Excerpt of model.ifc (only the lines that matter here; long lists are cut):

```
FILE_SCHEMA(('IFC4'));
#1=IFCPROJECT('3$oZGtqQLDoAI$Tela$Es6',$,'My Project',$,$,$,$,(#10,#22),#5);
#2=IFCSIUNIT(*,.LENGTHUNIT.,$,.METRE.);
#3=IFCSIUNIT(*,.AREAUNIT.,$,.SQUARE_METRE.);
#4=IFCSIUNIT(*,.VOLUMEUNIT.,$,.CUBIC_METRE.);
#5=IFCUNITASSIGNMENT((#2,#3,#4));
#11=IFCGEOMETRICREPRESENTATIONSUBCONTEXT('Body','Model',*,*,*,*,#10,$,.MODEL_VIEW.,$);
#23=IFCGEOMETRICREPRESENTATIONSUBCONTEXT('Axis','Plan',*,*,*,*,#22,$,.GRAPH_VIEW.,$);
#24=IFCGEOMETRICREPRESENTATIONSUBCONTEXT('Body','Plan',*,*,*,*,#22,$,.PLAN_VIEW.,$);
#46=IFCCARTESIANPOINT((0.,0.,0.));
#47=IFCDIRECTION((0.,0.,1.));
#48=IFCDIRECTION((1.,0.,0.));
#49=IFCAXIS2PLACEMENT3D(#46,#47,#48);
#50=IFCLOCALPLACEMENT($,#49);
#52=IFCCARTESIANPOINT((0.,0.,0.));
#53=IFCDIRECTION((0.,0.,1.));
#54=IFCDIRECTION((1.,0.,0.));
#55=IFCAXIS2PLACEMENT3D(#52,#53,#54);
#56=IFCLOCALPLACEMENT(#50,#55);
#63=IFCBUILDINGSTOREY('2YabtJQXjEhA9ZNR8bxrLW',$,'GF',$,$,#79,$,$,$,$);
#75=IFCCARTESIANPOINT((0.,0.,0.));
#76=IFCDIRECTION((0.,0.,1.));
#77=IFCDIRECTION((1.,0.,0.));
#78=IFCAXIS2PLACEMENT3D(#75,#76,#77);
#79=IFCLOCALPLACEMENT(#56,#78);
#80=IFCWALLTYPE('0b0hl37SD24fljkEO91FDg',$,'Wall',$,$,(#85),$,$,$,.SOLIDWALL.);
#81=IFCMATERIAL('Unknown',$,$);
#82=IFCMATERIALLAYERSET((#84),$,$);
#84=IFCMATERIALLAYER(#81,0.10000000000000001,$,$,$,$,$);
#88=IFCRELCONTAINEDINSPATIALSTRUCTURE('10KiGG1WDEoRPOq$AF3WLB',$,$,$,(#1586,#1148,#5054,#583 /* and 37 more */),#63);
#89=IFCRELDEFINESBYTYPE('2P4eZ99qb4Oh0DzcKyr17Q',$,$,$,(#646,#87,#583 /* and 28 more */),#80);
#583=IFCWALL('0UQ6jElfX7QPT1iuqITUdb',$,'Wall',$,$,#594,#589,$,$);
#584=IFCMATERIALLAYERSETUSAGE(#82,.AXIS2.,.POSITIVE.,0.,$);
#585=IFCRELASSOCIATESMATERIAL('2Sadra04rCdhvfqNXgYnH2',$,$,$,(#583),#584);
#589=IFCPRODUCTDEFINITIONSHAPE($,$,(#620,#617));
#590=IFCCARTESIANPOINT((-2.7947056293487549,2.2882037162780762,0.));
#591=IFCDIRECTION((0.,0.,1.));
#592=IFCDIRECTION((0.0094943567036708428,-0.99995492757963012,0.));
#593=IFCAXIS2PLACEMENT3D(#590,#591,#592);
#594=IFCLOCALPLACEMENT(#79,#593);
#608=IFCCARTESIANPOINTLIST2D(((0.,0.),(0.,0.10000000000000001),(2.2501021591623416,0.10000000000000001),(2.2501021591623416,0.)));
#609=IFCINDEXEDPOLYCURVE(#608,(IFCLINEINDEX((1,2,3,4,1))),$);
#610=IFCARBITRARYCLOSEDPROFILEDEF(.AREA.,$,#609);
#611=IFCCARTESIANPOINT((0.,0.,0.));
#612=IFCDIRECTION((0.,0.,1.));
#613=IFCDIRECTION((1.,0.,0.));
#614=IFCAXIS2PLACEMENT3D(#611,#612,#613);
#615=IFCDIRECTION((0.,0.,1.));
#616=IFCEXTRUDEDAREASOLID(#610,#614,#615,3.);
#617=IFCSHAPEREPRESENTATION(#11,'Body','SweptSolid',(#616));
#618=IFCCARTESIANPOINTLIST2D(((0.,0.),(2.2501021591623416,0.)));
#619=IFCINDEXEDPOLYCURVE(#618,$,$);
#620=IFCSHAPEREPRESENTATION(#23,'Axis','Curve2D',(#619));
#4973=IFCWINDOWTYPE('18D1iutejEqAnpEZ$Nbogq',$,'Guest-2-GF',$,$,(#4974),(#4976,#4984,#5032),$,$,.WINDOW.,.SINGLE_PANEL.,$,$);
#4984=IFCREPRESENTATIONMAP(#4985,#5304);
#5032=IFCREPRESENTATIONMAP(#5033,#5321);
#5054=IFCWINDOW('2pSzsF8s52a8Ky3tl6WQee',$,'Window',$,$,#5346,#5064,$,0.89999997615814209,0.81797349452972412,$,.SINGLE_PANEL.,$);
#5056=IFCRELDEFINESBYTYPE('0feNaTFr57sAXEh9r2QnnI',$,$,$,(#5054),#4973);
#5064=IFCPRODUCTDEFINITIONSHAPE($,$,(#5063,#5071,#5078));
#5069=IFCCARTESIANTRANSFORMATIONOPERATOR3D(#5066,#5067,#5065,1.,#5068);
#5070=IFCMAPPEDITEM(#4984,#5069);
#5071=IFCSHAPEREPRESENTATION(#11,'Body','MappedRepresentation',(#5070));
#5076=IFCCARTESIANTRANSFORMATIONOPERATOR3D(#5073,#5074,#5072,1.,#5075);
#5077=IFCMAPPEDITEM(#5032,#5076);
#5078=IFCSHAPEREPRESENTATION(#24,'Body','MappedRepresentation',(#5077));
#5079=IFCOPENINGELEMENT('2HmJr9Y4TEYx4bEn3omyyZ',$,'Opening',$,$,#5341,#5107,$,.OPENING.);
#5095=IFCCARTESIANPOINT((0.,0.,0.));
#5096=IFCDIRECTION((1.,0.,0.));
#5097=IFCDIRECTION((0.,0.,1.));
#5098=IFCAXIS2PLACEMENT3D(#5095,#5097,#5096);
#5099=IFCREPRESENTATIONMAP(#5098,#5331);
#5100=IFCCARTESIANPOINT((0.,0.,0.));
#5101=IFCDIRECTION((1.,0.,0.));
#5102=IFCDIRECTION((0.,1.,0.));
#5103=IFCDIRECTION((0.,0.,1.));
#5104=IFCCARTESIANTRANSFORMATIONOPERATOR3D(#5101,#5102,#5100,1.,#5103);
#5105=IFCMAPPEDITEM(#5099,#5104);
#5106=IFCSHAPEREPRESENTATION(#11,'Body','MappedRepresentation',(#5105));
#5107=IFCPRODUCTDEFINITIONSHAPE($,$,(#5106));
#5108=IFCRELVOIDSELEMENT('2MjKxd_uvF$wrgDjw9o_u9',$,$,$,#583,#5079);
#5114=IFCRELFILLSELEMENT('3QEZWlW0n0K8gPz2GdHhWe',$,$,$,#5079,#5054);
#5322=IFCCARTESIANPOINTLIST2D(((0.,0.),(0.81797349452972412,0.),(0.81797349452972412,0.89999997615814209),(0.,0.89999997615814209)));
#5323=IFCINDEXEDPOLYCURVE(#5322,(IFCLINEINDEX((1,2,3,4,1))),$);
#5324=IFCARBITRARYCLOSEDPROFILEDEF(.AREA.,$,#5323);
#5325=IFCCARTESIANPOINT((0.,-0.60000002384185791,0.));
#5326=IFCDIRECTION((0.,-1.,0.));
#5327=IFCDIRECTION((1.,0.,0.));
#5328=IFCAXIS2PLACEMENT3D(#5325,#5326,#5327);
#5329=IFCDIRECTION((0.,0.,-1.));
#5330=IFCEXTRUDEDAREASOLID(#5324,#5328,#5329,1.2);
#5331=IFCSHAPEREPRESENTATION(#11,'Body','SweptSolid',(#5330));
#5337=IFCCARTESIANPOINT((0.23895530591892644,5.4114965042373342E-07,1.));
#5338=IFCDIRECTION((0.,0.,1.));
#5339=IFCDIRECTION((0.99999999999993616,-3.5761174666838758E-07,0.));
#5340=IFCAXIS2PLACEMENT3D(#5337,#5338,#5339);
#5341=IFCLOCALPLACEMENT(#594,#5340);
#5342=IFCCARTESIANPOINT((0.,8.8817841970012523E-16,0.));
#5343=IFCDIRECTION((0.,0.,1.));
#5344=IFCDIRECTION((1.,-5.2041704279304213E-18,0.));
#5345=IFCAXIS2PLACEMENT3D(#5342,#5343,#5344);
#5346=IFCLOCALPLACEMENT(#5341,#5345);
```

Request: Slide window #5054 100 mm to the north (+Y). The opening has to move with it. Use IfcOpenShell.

```python
import ifcopenshell
import ifcopenshell.api.geometry
import ifcopenshell.util.placement

model = ifcopenshell.open("model.ifc")

window = model.by_guid("2pSzsF8s52a8Ky3tl6WQee")
opening = window.FillsVoids[0].RelatingOpeningElement
wall = opening.VoidsElements[0].RelatingBuildingElement

wall_matrix = ifcopenshell.util.placement.get_local_placement(wall.ObjectPlacement)
shift = wall_matrix[:3, 0] * -0.1
before = ifcopenshell.util.placement.get_local_placement(window.ObjectPlacement)[:3, 3].copy()

# The window is placed relative to its opening, so it follows when the opening moves.
matrix = ifcopenshell.util.placement.get_local_placement(opening.ObjectPlacement)
matrix[:3, 3] += shift
ifcopenshell.api.geometry.edit_object_placement(
    model, product=opening, matrix=matrix, is_si=False, should_transform_children=True
)

after = ifcopenshell.util.placement.get_local_placement(window.ObjectPlacement)[:3, 3]
print("window moved by", (after - before).round(3) + 0.0)

model.write("model_rev.ifc")
```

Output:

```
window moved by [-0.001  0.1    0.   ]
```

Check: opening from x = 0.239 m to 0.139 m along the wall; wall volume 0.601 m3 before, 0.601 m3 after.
